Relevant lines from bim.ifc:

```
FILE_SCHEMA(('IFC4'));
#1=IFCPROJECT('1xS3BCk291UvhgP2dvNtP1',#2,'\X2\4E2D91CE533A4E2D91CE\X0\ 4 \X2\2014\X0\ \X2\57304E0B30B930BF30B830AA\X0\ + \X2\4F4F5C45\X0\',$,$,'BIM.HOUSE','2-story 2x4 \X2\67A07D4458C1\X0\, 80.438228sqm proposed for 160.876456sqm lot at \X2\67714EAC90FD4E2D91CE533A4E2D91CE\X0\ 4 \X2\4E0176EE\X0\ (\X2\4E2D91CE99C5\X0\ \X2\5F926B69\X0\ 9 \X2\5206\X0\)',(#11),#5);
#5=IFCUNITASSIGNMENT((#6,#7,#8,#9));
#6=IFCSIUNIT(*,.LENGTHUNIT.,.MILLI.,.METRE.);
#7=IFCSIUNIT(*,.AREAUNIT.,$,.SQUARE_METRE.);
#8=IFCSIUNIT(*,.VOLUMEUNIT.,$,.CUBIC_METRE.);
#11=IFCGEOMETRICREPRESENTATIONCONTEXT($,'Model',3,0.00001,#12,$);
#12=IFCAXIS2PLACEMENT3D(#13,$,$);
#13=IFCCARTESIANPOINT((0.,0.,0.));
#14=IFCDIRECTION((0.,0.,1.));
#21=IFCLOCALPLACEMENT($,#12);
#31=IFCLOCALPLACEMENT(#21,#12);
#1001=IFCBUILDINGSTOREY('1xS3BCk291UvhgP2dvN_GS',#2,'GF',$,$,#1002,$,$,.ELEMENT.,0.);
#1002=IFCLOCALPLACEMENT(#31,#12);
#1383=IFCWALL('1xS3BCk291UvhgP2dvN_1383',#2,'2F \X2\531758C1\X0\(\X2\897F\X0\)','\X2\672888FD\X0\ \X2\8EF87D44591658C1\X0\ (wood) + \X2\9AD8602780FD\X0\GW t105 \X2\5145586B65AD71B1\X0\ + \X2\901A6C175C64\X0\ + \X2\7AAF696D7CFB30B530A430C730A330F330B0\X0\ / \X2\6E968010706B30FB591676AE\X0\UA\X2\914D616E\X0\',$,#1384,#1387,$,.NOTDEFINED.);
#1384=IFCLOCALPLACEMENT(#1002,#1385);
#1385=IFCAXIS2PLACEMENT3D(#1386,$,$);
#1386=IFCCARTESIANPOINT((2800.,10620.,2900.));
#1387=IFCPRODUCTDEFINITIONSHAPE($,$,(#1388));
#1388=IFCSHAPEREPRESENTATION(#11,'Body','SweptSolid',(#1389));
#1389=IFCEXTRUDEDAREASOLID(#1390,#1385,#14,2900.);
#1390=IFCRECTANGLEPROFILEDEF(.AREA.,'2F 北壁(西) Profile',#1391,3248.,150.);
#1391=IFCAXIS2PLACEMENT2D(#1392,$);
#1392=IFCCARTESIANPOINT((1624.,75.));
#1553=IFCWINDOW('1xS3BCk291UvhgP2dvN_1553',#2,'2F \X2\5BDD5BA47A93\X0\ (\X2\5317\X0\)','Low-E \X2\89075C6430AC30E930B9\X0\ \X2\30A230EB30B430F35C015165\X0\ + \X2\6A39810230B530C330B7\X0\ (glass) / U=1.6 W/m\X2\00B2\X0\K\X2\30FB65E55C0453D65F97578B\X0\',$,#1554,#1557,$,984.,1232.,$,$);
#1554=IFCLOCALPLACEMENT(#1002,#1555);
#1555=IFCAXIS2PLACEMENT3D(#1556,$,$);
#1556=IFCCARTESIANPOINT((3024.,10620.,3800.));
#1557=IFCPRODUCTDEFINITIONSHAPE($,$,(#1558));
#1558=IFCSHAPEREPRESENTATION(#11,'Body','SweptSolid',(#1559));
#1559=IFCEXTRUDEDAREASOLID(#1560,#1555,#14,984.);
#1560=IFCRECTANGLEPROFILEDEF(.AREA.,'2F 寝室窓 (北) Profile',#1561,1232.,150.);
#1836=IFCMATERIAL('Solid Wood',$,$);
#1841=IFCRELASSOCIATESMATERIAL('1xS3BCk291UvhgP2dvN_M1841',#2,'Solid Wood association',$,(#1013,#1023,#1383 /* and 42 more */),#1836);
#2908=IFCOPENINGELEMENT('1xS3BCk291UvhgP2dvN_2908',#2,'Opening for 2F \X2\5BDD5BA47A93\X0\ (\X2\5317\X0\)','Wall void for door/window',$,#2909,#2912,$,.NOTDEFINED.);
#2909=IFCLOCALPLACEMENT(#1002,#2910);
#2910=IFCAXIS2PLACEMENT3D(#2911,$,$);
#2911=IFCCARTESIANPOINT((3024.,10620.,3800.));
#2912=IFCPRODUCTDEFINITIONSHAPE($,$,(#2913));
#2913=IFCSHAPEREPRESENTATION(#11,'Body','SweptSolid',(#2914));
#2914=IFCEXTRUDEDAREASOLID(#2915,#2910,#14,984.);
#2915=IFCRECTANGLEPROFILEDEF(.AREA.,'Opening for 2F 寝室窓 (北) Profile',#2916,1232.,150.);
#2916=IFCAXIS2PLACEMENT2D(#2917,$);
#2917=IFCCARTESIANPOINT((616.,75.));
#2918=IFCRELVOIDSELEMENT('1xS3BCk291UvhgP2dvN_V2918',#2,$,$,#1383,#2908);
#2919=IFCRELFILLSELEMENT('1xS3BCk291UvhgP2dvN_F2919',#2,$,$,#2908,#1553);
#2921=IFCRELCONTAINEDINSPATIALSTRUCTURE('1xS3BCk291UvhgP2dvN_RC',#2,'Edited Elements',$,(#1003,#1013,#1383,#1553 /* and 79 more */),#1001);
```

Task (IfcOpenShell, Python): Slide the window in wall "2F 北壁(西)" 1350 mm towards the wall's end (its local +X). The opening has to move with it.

```python
import ifcopenshell
import ifcopenshell.api.geometry
import ifcopenshell.util.placement
import ifcopenshell.util.unit

model = ifcopenshell.open("bim.ifc")
unit_scale = ifcopenshell.util.unit.calculate_unit_scale(model)

window = model.by_id(1553)
opening = window.FillsVoids[0].RelatingOpeningElement
wall = opening.VoidsElements[0].RelatingBuildingElement

wall_matrix = ifcopenshell.util.placement.get_local_placement(wall.ObjectPlacement)
shift = wall_matrix[:3, 0] * 1.35 / unit_scale
before = ifcopenshell.util.placement.get_local_placement(window.ObjectPlacement)[:3, 3].copy()

# The window is not placed relative to its opening, so move both.
for product in (opening, window):
    matrix = ifcopenshell.util.placement.get_local_placement(product.ObjectPlacement)
    matrix[:3, 3] += shift
    ifcopenshell.api.geometry.edit_object_placement(model, product=product, matrix=matrix, is_si=False)

after = ifcopenshell.util.placement.get_local_placement(window.ObjectPlacement)[:3, 3]
print("window moved by", (after - before).round(3) + 0.0)

model.write("bim_updated.ifc")
```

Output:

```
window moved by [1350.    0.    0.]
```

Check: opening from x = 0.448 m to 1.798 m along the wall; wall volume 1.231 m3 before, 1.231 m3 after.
